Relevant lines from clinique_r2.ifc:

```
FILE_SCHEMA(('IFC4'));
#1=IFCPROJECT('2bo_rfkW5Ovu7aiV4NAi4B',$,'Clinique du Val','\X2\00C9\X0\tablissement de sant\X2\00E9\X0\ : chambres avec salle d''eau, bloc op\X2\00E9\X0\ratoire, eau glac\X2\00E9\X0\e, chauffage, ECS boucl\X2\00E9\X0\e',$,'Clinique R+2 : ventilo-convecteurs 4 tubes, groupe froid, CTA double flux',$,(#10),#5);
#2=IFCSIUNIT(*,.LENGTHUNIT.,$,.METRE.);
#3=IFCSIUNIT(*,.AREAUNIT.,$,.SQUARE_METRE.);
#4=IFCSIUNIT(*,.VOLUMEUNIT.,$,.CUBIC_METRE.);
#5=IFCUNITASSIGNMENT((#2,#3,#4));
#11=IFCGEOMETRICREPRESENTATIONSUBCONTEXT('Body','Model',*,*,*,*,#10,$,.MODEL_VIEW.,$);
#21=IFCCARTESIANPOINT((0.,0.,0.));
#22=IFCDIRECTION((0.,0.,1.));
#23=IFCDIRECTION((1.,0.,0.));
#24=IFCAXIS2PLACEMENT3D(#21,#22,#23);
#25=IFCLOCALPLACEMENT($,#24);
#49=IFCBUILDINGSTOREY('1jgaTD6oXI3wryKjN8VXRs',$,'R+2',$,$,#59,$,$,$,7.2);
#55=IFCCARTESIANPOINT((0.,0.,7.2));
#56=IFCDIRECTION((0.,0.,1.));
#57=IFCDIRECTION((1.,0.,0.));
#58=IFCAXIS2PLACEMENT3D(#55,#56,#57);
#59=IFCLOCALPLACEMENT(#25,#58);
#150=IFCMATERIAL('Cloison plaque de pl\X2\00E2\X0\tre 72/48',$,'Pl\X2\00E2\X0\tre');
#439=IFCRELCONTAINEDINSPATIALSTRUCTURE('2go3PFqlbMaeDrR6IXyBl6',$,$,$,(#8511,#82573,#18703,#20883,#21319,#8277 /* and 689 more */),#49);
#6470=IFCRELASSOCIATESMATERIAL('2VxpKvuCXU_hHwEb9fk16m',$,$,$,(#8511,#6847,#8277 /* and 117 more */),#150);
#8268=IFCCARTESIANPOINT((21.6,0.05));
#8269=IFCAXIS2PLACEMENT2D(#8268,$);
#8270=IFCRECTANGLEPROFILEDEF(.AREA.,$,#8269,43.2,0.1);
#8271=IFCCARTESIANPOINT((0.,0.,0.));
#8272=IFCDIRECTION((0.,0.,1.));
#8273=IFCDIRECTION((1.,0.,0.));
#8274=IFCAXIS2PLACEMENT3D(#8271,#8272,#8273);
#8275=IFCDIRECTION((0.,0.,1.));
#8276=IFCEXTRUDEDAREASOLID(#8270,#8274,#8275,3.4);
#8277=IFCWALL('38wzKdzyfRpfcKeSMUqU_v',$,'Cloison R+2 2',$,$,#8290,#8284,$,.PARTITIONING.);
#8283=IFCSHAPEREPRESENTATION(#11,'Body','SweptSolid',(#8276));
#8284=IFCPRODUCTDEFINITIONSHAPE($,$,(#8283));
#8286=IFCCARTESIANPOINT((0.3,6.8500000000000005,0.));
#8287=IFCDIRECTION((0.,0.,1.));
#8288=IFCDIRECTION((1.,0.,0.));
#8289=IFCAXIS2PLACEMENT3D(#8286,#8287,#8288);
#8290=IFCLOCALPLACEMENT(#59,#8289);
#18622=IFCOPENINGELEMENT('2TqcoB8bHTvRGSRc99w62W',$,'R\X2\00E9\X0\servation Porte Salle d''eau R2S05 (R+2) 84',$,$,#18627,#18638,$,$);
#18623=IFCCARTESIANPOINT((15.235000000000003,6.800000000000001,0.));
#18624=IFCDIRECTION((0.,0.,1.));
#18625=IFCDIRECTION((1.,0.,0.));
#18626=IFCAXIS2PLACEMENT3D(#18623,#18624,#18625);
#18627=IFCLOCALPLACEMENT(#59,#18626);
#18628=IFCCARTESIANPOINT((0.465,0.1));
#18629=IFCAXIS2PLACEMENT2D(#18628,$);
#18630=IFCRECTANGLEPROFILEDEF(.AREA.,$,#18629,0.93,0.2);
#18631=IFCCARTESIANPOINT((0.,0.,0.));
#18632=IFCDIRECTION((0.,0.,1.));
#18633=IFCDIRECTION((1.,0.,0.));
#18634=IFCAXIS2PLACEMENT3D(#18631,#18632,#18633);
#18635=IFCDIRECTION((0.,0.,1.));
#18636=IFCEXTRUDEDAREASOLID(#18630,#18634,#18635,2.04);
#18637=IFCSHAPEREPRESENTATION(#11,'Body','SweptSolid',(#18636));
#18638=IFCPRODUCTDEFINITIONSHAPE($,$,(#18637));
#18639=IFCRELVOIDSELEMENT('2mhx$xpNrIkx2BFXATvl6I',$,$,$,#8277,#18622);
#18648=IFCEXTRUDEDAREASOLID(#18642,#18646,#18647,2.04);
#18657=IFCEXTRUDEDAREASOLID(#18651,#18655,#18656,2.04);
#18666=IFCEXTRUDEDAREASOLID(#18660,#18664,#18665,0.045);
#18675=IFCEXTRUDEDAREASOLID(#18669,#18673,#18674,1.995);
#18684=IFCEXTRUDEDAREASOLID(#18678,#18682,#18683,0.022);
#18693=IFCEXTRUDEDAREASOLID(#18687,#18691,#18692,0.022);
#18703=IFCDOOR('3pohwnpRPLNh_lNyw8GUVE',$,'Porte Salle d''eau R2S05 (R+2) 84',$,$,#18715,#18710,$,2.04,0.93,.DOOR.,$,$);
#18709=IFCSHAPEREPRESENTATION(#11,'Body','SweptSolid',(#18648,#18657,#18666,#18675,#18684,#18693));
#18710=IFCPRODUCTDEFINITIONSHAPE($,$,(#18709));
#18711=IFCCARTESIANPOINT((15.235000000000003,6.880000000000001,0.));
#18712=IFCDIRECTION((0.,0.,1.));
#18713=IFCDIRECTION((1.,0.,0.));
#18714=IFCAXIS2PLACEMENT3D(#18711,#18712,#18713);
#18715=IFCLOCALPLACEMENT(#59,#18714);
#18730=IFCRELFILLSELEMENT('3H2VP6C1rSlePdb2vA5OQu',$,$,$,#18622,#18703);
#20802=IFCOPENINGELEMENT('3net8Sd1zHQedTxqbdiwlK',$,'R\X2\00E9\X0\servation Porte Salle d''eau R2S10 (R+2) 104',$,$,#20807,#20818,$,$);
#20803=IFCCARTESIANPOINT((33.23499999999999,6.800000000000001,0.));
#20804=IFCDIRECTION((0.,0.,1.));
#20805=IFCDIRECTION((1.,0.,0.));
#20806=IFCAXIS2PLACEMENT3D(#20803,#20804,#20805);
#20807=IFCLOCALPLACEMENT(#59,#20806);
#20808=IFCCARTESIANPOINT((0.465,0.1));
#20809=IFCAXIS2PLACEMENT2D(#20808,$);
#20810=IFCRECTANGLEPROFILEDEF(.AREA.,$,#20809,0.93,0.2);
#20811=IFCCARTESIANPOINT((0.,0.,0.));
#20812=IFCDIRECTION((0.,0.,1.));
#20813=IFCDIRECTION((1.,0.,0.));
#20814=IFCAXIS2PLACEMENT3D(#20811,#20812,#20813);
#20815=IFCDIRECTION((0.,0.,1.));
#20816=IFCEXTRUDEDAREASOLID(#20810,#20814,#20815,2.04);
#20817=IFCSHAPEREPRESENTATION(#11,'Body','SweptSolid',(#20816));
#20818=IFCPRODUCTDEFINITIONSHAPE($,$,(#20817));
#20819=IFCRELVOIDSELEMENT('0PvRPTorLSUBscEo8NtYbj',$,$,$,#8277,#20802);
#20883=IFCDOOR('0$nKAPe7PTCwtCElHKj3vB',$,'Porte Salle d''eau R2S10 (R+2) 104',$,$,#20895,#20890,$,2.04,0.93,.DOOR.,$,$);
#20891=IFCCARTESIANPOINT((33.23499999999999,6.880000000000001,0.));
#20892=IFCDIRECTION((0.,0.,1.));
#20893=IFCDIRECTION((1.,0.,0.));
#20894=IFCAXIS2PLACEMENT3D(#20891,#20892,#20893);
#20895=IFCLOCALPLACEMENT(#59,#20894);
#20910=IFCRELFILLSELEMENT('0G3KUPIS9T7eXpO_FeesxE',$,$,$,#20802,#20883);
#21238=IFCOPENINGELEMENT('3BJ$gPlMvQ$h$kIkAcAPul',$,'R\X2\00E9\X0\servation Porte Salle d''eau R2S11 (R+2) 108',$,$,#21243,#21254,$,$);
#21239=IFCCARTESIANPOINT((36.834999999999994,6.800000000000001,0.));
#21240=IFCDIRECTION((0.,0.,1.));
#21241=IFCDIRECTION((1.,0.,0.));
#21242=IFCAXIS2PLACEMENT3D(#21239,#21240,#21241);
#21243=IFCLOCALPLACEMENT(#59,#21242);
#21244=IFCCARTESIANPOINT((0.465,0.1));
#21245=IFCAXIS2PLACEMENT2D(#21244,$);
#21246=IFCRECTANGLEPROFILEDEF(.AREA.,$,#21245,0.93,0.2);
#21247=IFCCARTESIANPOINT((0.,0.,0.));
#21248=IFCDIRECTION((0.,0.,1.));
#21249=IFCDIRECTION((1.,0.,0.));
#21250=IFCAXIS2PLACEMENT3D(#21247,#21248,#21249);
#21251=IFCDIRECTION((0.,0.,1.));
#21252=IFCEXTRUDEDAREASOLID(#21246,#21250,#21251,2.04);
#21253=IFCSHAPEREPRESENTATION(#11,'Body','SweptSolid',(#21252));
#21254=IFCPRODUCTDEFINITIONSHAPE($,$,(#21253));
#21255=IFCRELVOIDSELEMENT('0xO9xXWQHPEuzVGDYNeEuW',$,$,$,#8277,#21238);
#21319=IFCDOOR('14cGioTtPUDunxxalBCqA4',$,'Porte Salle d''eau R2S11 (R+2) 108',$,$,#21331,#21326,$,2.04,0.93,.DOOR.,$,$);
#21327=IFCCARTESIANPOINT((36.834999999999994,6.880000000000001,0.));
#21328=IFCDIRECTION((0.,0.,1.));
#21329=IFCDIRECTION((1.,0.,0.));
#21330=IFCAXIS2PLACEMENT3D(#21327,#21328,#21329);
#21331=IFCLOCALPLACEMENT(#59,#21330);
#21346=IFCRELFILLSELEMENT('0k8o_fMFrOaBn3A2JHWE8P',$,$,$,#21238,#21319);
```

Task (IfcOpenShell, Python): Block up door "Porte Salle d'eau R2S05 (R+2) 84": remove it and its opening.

```python
import ifcopenshell
import ifcopenshell.api.feature
import ifcopenshell.api.root
import ifcopenshell.geom
import ifcopenshell.util.shape

model = ifcopenshell.open("clinique_r2.ifc")
settings = ifcopenshell.geom.settings()


def volume(element):
    """Net volume in cubic metres, openings subtracted."""
    shape = ifcopenshell.geom.create_shape(settings, element)
    return ifcopenshell.util.shape.get_volume(shape.geometry)


door = model.by_guid("3pohwnpRPLNh_lNyw8GUVE")
opening = door.FillsVoids[0].RelatingOpeningElement
wall = opening.VoidsElements[0].RelatingBuildingElement
before = volume(wall)

ifcopenshell.api.root.remove_product(model, product=door)
ifcopenshell.api.feature.remove_feature(model, feature=opening)

after = volume(wall)

print(f"wall volume {before:.3f} -> {after:.3f} m3")

model.write("clinique_r2-out.ifc")
```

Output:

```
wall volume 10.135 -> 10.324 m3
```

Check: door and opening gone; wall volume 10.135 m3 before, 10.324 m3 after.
